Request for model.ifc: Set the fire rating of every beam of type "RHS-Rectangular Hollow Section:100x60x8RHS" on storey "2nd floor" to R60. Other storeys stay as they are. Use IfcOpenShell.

First a look at what the model holds.

```python
import ifcopenshell
import ifcopenshell.util.element

model = ifcopenshell.open("model.ifc")
print(model.schema)
storey = next(s for s in model.by_type("IfcBuildingStorey") if s.Name == "2nd floor")
beams = [e for e in ifcopenshell.util.element.get_decomposition(storey) if e.is_a("IfcBeam")]
seen = {}
for e in beams:
    element_type = ifcopenshell.util.element.get_type(e)
    key = (element_type.Name if element_type != e and element_type else None, ifcopenshell.util.element.get_pset(e, "Pset_BeamCommon", "FireRating"))
    seen[key] = seen.get(key, 0) + 1
for (name, value), count in sorted(seen.items(), key=str):
    print(count, "x", name, "|", value)
```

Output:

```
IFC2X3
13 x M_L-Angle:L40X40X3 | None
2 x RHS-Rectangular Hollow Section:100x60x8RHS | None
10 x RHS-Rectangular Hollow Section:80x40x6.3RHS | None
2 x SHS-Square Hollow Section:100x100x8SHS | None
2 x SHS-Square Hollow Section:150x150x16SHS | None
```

```python
import ifcopenshell
import ifcopenshell.api.pset
import ifcopenshell.util.element

model = ifcopenshell.open("model.ifc")

storey = next(s for s in model.by_type("IfcBuildingStorey") if s.Name == "2nd floor")
beams = [e for e in ifcopenshell.util.element.get_decomposition(storey) if e.is_a("IfcBeam")]

count = 0
for e in beams:
    element_type = ifcopenshell.util.element.get_type(e)
    if element_type in (None, e) or element_type.Name != "RHS-Rectangular Hollow Section:100x60x8RHS":
        continue
    # add_pset returns the element's existing set when there is one.
    pset = ifcopenshell.api.pset.add_pset(model, product=e, name="Pset_BeamCommon")
    ifcopenshell.api.pset.edit_pset(model, pset=pset, properties={"FireRating": "R60"})
    count += 1

print(count, "beams updated")

model.write("model_edited.ifc")
```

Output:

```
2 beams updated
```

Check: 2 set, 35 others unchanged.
